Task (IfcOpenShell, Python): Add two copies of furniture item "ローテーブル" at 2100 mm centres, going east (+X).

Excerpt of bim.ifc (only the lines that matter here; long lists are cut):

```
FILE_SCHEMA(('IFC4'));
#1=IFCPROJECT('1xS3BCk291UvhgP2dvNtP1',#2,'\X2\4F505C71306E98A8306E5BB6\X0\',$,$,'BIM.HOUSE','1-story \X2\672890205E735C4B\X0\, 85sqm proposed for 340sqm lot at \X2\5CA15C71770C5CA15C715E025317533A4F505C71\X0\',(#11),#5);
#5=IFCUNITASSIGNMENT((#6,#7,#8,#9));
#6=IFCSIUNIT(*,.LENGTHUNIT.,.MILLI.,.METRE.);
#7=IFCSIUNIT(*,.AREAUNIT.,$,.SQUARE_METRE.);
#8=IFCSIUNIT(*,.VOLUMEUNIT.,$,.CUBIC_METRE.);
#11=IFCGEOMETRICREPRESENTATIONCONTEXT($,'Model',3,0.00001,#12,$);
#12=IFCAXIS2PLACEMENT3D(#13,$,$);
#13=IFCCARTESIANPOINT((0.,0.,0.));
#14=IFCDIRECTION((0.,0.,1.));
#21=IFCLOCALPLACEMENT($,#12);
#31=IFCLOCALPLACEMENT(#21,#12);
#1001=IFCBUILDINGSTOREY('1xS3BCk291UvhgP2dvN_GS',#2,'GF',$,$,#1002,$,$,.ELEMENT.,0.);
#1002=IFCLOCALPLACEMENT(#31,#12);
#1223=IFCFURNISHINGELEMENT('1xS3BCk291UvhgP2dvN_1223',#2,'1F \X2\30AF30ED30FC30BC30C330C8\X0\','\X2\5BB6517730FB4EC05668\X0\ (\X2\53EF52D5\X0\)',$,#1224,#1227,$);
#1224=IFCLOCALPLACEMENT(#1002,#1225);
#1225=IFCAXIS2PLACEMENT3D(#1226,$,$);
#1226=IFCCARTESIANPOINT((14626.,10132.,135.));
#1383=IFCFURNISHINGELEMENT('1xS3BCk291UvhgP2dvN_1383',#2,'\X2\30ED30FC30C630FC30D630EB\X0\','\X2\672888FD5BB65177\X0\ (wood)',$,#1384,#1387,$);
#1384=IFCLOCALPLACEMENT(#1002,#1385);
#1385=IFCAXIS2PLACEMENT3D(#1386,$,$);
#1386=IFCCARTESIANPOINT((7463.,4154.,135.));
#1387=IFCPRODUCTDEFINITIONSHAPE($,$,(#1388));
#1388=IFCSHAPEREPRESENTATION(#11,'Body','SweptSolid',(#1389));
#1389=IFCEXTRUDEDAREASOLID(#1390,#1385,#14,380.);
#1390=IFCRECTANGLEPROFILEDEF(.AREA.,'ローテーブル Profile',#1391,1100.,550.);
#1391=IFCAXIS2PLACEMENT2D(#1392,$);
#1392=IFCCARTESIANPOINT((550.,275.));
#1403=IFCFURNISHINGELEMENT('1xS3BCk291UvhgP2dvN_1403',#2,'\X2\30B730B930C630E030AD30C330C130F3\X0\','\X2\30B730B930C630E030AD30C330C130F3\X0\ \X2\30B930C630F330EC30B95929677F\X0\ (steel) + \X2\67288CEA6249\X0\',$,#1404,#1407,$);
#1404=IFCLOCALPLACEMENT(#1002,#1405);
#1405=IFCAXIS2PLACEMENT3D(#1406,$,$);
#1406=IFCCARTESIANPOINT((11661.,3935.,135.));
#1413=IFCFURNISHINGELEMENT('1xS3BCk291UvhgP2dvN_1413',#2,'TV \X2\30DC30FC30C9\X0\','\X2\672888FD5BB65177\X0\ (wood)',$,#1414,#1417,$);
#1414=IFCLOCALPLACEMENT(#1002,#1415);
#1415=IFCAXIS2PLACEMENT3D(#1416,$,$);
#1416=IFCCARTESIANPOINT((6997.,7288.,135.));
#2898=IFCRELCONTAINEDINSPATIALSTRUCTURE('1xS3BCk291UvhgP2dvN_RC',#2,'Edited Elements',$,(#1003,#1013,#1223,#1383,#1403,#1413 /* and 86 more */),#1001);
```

```python
import numpy as np
import ifcopenshell
import ifcopenshell.api.geometry
import ifcopenshell.api.root
import ifcopenshell.util.element
import ifcopenshell.util.placement

model = ifcopenshell.open("bim.ifc")


def reuse_history(source, copy):
    """copy_class also copies each property set's owner history, people and application; keep the originals."""
    for rel in copy.IsDefinedBy:
        if rel.is_a("IfcRelDefinesByProperties") and (history := rel.RelatingPropertyDefinition.OwnerHistory):
            rel.RelatingPropertyDefinition.OwnerHistory = source.OwnerHistory
            ifcopenshell.util.element.remove_deep2(model, history)


source = model.by_guid("1xS3BCk291UvhgP2dvN_1383")
base = ifcopenshell.util.placement.get_local_placement(source.ObjectPlacement)
step = np.array([1.0, 0.0, 0.0]) * 2100.0

for i in range(1, 3):
    copy = ifcopenshell.api.root.copy_class(model, product=source)
    copy.Representation = ifcopenshell.util.element.copy_deep(
        model, source.Representation, exclude=["IfcGeometricRepresentationContext", "IfcRepresentationMap"]
    )
    reuse_history(source, copy)
    matrix = base.copy()
    matrix[:3, 3] += i * step
    print("added at", matrix[:3, 3].round(3) + 0.0)
    ifcopenshell.api.geometry.edit_object_placement(model, product=copy, matrix=matrix, is_si=False)

model.write("bim_updated.ifc")
```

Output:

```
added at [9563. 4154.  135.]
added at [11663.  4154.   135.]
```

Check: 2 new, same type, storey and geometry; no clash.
